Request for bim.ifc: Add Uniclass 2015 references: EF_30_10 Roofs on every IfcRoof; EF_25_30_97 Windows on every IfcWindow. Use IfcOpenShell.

First a look at what the model holds.

```python
import ifcopenshell

model = ifcopenshell.open("bim.ifc")
print(model.schema)
print("classifications:", [c.Name for c in model.by_type("IfcClassification")])
for ifc_class in ("IfcDoor", "IfcRoof", "IfcStair", "IfcWall", "IfcWindow"):
    print(ifc_class, len(model.by_type(ifc_class)))
```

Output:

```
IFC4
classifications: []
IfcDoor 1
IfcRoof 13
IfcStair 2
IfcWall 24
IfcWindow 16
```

```python
import ifcopenshell
import ifcopenshell.api.classification

model = ifcopenshell.open("bim.ifc")

system = ifcopenshell.api.classification.add_classification(model, classification="Uniclass 2015")

codes = {
    "IfcRoof": ("EF_30_10", "Roofs"),
    "IfcWindow": ("EF_25_30_97", "Windows"),
}
for ifc_class, (code, name) in codes.items():
    products = model.by_type(ifc_class)
    ifcopenshell.api.classification.add_reference(
        model, products=products, classification=system, identification=code, name=name
    )
    print(code, len(products))

model.write("bim_rev.ifc")
```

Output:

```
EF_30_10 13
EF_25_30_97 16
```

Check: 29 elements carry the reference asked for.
